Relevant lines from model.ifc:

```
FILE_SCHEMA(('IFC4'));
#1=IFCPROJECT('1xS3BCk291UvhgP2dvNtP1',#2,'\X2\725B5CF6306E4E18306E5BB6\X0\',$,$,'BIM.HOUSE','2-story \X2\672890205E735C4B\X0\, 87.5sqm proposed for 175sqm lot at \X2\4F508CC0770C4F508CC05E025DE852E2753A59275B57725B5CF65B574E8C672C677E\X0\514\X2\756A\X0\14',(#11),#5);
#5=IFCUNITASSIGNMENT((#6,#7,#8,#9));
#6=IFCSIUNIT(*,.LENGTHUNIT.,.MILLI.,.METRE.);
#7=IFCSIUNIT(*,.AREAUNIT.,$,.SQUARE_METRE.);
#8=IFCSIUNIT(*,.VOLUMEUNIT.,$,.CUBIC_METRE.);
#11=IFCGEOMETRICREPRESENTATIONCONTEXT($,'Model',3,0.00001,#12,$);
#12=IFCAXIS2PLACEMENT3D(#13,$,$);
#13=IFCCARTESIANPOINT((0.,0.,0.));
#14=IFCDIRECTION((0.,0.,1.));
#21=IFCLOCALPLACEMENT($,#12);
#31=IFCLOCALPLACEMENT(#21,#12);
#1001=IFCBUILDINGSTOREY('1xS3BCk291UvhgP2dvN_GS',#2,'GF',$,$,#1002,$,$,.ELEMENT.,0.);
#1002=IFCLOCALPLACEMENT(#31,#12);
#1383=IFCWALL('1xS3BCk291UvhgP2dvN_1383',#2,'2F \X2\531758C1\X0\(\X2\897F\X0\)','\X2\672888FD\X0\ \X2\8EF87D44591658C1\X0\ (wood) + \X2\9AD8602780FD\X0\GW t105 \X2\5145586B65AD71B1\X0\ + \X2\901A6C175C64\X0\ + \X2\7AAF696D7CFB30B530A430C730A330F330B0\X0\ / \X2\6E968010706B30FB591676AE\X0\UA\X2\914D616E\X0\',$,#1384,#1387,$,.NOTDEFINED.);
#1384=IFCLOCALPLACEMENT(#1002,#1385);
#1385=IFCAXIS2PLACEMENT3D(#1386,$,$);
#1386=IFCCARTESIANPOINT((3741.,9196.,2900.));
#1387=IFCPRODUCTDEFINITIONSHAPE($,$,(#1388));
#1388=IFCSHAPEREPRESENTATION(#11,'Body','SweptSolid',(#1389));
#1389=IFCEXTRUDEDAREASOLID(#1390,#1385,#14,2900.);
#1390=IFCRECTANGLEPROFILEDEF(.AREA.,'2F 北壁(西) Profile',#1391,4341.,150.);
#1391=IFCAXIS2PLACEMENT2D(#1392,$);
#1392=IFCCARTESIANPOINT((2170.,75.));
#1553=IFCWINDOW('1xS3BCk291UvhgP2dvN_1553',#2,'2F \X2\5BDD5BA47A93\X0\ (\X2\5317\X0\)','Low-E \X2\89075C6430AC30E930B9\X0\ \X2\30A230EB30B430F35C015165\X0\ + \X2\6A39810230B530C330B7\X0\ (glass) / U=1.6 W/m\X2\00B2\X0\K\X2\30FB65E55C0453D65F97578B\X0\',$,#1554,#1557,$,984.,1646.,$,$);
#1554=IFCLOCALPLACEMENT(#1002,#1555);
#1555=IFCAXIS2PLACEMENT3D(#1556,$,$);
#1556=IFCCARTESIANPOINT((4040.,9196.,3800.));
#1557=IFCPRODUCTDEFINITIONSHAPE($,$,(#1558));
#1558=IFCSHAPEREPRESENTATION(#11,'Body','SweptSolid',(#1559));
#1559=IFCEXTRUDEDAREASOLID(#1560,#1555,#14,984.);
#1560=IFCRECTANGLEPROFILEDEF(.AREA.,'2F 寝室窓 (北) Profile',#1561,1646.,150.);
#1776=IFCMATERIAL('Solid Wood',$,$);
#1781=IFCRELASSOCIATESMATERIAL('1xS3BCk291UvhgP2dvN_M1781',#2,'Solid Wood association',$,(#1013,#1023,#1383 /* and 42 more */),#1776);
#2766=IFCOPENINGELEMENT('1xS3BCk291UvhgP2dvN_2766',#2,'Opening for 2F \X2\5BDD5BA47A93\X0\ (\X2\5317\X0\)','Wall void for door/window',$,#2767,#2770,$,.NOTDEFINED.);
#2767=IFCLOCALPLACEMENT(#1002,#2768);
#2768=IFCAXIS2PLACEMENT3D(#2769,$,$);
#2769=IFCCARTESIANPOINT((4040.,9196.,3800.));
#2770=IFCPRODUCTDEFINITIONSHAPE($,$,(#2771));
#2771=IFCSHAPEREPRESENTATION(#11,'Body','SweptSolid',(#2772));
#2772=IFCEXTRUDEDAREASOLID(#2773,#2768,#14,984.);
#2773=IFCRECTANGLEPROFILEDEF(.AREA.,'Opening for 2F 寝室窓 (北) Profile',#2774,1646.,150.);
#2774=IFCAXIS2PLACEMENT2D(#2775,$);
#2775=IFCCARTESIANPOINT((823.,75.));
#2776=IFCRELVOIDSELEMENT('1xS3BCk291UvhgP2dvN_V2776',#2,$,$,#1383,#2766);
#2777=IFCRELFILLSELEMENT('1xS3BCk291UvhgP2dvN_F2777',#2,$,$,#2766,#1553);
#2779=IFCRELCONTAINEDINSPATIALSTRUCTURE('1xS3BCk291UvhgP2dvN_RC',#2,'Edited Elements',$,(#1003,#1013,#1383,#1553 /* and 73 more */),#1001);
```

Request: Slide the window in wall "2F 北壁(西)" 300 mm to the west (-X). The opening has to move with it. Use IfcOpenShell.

```python
import ifcopenshell
import ifcopenshell.api.geometry
import ifcopenshell.util.placement
import ifcopenshell.util.unit

model = ifcopenshell.open("model.ifc")
unit_scale = ifcopenshell.util.unit.calculate_unit_scale(model)

window = model.by_guid("1xS3BCk291UvhgP2dvN_1553")
opening = window.FillsVoids[0].RelatingOpeningElement
wall = opening.VoidsElements[0].RelatingBuildingElement

wall_matrix = ifcopenshell.util.placement.get_local_placement(wall.ObjectPlacement)
shift = wall_matrix[:3, 0] * -0.3 / unit_scale
before = ifcopenshell.util.placement.get_local_placement(window.ObjectPlacement)[:3, 3].copy()

# The window is not placed relative to its opening, so move both.
for product in (opening, window):
    matrix = ifcopenshell.util.placement.get_local_placement(product.ObjectPlacement)
    matrix[:3, 3] += shift
    ifcopenshell.api.geometry.edit_object_placement(model, product=product, matrix=matrix, is_si=False)

after = ifcopenshell.util.placement.get_local_placement(window.ObjectPlacement)[:3, 3]
print("window moved by", (after - before).round(3) + 0.0)

model.write("model_rev.ifc")
```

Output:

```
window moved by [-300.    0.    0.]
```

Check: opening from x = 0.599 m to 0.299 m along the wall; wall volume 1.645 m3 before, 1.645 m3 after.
